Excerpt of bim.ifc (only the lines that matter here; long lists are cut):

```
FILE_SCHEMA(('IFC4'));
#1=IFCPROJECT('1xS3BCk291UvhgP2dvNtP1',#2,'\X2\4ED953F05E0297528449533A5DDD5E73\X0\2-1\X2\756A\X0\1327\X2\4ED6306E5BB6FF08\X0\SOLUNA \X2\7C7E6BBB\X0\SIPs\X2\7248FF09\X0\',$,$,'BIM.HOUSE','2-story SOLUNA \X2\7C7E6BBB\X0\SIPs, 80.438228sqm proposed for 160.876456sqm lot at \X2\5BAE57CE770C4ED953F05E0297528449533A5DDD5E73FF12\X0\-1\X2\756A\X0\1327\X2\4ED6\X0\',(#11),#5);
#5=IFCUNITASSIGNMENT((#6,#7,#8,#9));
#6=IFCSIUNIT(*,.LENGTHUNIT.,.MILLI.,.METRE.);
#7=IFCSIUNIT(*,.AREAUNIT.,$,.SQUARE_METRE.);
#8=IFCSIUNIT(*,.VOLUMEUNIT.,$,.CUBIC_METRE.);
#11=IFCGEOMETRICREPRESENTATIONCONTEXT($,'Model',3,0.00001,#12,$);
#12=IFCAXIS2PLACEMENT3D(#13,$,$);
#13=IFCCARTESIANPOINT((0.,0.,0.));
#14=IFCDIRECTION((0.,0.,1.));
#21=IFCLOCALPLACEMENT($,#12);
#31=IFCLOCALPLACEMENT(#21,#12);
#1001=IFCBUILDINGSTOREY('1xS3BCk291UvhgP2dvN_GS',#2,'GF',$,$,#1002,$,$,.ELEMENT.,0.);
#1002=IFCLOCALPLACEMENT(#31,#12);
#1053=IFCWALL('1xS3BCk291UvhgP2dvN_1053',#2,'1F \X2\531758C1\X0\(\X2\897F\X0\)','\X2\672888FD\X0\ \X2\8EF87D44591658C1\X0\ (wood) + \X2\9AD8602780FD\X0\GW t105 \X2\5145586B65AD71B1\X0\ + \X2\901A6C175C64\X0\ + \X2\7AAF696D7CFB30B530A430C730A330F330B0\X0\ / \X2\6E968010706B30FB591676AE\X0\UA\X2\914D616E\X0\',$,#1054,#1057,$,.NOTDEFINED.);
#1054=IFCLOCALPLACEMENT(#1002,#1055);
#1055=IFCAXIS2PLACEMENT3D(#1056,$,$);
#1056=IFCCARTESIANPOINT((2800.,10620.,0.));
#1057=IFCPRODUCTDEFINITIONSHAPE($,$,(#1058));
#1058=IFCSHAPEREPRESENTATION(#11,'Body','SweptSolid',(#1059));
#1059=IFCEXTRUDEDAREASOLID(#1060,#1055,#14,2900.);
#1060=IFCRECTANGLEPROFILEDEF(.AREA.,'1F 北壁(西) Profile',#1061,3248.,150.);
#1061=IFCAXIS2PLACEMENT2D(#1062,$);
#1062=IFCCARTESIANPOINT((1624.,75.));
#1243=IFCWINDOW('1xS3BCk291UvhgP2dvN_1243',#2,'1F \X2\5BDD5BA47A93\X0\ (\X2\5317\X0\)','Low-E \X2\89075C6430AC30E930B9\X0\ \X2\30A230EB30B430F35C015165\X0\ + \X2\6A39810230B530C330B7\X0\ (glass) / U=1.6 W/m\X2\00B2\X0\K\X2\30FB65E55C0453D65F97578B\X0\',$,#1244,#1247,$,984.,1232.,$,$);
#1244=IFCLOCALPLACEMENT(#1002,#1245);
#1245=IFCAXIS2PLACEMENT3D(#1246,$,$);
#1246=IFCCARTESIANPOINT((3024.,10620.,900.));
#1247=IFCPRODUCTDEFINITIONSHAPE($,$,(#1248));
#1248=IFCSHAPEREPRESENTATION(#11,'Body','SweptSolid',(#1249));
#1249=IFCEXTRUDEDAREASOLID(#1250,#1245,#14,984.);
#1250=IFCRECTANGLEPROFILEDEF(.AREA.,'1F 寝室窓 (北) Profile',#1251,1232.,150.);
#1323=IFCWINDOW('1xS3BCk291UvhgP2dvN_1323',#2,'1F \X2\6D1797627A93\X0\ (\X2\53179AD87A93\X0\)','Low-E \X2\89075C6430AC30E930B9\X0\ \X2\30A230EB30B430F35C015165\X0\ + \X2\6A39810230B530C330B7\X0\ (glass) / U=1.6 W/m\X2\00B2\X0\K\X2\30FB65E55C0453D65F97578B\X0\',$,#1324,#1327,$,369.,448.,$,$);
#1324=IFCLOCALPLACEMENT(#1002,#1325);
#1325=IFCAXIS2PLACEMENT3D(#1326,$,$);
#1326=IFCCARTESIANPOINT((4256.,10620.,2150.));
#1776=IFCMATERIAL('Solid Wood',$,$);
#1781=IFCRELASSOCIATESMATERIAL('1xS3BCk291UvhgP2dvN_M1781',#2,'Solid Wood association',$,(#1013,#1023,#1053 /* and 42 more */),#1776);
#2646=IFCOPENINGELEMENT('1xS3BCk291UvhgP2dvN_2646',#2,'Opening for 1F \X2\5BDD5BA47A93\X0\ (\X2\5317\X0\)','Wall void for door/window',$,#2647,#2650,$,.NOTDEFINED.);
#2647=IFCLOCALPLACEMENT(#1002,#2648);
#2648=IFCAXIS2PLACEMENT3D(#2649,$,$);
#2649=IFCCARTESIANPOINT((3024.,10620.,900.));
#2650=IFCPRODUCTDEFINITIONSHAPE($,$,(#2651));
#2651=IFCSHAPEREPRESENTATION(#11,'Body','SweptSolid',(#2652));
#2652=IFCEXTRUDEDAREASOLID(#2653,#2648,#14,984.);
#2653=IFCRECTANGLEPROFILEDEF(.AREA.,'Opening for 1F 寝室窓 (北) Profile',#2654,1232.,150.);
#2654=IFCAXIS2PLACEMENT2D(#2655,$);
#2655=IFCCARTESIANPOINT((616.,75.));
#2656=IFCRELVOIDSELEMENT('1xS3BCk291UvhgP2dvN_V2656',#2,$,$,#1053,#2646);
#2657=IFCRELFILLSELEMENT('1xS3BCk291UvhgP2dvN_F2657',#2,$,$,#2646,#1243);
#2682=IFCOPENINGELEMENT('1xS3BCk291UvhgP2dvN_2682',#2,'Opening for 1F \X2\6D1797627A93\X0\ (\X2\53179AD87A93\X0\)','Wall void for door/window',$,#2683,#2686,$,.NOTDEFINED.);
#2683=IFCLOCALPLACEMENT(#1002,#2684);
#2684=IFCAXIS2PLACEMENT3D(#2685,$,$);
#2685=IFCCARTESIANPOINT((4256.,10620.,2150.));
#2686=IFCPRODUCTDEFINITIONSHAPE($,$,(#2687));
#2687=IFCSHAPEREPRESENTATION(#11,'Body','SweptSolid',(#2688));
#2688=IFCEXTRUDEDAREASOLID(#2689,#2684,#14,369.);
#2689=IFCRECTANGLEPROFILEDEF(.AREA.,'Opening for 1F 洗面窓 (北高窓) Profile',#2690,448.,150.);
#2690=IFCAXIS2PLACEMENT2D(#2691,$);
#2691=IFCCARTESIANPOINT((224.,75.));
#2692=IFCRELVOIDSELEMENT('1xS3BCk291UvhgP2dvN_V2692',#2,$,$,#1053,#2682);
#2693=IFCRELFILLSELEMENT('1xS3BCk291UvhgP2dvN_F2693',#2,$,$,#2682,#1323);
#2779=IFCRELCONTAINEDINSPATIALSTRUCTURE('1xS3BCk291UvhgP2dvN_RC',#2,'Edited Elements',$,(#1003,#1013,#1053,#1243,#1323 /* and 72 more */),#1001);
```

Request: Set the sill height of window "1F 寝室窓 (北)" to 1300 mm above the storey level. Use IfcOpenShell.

```python
import numpy as np
import ifcopenshell
import ifcopenshell.api.geometry
import ifcopenshell.geom
import ifcopenshell.util.element
import ifcopenshell.util.placement
import ifcopenshell.util.shape
import ifcopenshell.util.unit

model = ifcopenshell.open("bim.ifc")
unit_scale = ifcopenshell.util.unit.calculate_unit_scale(model)

window = model.by_guid("1xS3BCk291UvhgP2dvN_1243")
opening = window.FillsVoids[0].RelatingOpeningElement
storey = ifcopenshell.util.element.get_container(window, ifc_class="IfcBuildingStorey")
level = ifcopenshell.util.placement.get_local_placement(storey.ObjectPlacement)[2, 3]

# The opening's origin need not be at the sill, so measure its lowest point.
shape = ifcopenshell.geom.create_shape(ifcopenshell.geom.settings(), opening)
bottom = ifcopenshell.util.shape.get_shape_bottom_elevation(shape, shape.geometry) / unit_scale
dz = level + 1.3 / unit_scale - bottom

shift = np.array([0.0, 0.0, dz])
# The window is not placed relative to its opening, so move both.
for product in (opening, window):
    matrix = ifcopenshell.util.placement.get_local_placement(product.ObjectPlacement)
    matrix[:3, 3] += shift
    ifcopenshell.api.geometry.edit_object_placement(model, product=product, matrix=matrix, is_si=False)

print(f"moved by {dz * unit_scale:+.3f} m")

model.write("bim_edited.ifc")
```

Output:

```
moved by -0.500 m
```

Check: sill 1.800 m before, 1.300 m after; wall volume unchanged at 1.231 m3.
